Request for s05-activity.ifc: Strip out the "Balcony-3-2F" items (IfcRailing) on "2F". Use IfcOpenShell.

First a look at what the model holds.

```python
import ifcopenshell
import ifcopenshell.util.element

model = ifcopenshell.open("s05-activity.ifc")
print(model.schema)
storey = next(s for s in model.by_type("IfcBuildingStorey") if s.Name == "2F")
railings = [e for e in ifcopenshell.util.element.get_decomposition(storey) if e.is_a("IfcRailing")]
seen = {}
for e in railings:
    element_type = ifcopenshell.util.element.get_type(e)
    name = element_type.Name if element_type not in (None, e) else None
    seen[name] = seen.get(name, 0) + 1
for name, count in sorted(seen.items(), key=str):
    print(count, "x", name)
```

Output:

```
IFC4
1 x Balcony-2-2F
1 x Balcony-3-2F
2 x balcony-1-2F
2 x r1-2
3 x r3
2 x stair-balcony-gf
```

```python
import ifcopenshell
import ifcopenshell.api.root
import ifcopenshell.util.element

model = ifcopenshell.open("s05-activity.ifc")

storey = next(s for s in model.by_type("IfcBuildingStorey") if s.Name == "2F")
railings = [e for e in ifcopenshell.util.element.get_decomposition(storey) if e.is_a("IfcRailing")]
targets = [e for e in railings if (t := ifcopenshell.util.element.get_type(e)) not in (None, e) and t.Name == "Balcony-3-2F"]

for e in targets:
    ifcopenshell.api.root.remove_product(model, product=e)
print(len(targets), "removed")

model.write("s05-activity_rev.ifc")
```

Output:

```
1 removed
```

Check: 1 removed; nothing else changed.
